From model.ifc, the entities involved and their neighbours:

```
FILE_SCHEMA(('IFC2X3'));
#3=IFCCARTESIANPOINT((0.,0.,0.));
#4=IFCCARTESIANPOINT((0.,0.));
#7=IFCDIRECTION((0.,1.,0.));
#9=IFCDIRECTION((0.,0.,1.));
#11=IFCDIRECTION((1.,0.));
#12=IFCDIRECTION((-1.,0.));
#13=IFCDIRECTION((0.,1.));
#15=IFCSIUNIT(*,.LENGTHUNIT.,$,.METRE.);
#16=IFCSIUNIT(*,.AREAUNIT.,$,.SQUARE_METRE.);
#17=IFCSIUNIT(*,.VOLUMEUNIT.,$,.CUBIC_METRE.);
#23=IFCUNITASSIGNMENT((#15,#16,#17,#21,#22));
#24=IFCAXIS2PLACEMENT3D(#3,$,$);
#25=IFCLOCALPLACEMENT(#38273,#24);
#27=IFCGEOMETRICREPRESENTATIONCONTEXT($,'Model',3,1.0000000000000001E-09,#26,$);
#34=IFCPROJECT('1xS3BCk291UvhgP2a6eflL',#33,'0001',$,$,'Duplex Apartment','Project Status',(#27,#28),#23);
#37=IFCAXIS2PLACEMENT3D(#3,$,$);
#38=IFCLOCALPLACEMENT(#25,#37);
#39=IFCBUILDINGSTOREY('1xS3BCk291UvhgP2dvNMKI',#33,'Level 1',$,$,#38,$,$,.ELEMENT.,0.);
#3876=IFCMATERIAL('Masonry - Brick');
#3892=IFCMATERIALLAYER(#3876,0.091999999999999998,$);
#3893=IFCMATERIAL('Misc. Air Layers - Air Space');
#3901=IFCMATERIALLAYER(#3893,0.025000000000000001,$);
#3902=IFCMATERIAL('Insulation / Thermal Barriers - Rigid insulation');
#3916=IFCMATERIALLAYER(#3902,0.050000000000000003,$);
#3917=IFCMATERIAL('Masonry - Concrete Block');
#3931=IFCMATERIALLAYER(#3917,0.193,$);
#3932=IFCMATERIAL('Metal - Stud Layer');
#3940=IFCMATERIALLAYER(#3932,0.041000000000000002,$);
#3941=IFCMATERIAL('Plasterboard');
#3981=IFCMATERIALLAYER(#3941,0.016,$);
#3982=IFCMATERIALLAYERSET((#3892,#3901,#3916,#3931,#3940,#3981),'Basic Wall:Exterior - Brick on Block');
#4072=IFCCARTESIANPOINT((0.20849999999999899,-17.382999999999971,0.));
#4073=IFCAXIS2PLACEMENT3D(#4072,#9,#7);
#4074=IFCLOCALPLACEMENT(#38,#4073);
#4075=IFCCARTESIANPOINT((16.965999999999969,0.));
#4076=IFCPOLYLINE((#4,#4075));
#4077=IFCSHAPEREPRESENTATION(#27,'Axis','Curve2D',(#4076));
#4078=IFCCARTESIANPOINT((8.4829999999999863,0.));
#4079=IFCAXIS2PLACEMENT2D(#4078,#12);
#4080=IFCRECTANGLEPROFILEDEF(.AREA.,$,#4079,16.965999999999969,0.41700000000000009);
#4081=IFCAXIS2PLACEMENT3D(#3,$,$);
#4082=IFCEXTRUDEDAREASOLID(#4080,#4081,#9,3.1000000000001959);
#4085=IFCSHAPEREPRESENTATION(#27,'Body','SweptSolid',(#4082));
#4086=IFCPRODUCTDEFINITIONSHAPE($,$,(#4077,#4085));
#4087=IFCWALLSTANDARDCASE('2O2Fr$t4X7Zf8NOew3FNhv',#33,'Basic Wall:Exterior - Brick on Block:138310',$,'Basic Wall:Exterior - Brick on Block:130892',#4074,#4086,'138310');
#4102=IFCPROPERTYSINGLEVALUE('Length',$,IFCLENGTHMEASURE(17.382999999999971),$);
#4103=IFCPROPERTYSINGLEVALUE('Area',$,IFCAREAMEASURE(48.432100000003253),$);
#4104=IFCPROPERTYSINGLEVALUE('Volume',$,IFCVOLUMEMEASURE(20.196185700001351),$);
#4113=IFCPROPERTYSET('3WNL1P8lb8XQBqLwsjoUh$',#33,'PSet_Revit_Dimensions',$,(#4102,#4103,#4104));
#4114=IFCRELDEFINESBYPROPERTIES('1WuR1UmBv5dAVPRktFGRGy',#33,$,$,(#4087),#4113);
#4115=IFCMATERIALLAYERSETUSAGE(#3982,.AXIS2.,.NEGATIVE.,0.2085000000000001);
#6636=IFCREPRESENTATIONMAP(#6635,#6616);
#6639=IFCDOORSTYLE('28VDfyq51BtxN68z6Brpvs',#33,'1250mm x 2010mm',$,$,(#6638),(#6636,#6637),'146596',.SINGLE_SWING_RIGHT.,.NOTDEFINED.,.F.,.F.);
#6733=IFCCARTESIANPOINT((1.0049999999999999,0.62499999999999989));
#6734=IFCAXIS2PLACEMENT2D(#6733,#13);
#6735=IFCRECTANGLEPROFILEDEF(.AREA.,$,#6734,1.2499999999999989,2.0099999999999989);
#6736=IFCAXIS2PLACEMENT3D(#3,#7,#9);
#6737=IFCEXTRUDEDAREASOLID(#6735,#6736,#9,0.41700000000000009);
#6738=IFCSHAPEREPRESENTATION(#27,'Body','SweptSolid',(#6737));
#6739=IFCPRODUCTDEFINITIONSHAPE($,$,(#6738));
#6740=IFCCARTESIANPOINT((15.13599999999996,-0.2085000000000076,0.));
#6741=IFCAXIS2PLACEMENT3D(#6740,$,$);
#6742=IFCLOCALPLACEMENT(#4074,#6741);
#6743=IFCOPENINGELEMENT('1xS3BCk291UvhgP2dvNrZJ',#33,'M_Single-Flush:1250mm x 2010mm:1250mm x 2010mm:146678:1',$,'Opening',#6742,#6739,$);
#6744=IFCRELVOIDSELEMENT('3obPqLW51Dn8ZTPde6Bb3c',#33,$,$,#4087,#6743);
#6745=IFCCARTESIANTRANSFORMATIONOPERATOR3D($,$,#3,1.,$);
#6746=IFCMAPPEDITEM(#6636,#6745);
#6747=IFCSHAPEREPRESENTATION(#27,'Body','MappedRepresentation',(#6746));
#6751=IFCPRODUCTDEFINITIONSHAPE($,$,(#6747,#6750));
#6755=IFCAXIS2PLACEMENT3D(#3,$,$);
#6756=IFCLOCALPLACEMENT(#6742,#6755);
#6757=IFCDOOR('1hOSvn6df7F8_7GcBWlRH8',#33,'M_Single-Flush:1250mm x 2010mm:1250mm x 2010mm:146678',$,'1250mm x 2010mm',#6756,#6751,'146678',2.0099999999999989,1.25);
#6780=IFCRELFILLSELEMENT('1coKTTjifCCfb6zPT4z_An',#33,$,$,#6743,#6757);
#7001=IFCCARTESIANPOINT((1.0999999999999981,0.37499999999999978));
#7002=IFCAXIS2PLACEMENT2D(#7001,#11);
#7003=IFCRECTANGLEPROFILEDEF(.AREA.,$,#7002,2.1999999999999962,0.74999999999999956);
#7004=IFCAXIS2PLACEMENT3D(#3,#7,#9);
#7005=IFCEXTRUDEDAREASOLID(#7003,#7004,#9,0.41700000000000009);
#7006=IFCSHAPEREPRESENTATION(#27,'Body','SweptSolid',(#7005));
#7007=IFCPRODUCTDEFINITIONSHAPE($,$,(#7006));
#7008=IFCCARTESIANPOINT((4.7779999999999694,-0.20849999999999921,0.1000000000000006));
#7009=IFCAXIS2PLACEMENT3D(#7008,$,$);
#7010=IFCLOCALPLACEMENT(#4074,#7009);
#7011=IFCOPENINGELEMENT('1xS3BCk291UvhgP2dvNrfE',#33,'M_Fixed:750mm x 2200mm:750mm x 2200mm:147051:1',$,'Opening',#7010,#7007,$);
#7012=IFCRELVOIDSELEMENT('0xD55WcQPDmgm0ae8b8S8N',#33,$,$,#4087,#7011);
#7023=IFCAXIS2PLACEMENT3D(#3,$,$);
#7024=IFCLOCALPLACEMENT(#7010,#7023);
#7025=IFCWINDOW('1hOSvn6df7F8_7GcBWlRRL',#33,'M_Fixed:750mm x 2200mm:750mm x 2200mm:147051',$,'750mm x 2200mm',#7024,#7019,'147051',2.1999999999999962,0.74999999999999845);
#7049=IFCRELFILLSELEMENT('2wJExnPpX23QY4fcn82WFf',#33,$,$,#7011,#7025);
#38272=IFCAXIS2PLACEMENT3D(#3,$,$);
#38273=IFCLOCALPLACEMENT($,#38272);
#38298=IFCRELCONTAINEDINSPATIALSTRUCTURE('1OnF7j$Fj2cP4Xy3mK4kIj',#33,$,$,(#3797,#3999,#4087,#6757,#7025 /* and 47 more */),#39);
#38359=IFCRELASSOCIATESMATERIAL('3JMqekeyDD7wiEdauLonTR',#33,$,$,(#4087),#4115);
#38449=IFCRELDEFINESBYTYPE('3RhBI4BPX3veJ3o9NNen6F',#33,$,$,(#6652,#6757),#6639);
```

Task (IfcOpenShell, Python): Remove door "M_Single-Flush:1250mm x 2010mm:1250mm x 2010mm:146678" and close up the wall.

```python
import ifcopenshell
import ifcopenshell.api.feature
import ifcopenshell.api.pset
import ifcopenshell.api.root
import ifcopenshell.geom
import ifcopenshell.util.element
import ifcopenshell.util.shape
import ifcopenshell.util.unit

model = ifcopenshell.open("model.ifc")
area_scale = ifcopenshell.util.unit.calculate_unit_scale(model, "AREAUNIT")
volume_scale = ifcopenshell.util.unit.calculate_unit_scale(model, "VOLUMEUNIT")
settings = ifcopenshell.geom.settings()


def volume(element):
    """Net volume in cubic metres, openings subtracted."""
    shape = ifcopenshell.geom.create_shape(settings, element)
    return ifcopenshell.util.shape.get_volume(shape.geometry)


door = model.by_id(6757)
opening = door.FillsVoids[0].RelatingOpeningElement
wall = opening.VoidsElements[0].RelatingBuildingElement
before = volume(wall)

ifcopenshell.api.root.remove_product(model, product=door)
ifcopenshell.api.feature.remove_feature(model, feature=opening)

after = volume(wall)
thickness = 0.417  # wall thickness in metres

# Update the wall's stored quantities.
pset = model.by_id(ifcopenshell.util.element.get_pset(wall, "PSet_Revit_Dimensions", should_inherit=False)["id"])
ifcopenshell.api.pset.edit_pset(model, pset=pset, properties={
    "Area": model.create_entity("IfcAreaMeasure", after / thickness / area_scale),
    "Volume": model.create_entity("IfcVolumeMeasure", after / volume_scale),
})

print(f"wall volume {before:.3f} -> {after:.3f} m3")

model.write("model_edited.ifc")
```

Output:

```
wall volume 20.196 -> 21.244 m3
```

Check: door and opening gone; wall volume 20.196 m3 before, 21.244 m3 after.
